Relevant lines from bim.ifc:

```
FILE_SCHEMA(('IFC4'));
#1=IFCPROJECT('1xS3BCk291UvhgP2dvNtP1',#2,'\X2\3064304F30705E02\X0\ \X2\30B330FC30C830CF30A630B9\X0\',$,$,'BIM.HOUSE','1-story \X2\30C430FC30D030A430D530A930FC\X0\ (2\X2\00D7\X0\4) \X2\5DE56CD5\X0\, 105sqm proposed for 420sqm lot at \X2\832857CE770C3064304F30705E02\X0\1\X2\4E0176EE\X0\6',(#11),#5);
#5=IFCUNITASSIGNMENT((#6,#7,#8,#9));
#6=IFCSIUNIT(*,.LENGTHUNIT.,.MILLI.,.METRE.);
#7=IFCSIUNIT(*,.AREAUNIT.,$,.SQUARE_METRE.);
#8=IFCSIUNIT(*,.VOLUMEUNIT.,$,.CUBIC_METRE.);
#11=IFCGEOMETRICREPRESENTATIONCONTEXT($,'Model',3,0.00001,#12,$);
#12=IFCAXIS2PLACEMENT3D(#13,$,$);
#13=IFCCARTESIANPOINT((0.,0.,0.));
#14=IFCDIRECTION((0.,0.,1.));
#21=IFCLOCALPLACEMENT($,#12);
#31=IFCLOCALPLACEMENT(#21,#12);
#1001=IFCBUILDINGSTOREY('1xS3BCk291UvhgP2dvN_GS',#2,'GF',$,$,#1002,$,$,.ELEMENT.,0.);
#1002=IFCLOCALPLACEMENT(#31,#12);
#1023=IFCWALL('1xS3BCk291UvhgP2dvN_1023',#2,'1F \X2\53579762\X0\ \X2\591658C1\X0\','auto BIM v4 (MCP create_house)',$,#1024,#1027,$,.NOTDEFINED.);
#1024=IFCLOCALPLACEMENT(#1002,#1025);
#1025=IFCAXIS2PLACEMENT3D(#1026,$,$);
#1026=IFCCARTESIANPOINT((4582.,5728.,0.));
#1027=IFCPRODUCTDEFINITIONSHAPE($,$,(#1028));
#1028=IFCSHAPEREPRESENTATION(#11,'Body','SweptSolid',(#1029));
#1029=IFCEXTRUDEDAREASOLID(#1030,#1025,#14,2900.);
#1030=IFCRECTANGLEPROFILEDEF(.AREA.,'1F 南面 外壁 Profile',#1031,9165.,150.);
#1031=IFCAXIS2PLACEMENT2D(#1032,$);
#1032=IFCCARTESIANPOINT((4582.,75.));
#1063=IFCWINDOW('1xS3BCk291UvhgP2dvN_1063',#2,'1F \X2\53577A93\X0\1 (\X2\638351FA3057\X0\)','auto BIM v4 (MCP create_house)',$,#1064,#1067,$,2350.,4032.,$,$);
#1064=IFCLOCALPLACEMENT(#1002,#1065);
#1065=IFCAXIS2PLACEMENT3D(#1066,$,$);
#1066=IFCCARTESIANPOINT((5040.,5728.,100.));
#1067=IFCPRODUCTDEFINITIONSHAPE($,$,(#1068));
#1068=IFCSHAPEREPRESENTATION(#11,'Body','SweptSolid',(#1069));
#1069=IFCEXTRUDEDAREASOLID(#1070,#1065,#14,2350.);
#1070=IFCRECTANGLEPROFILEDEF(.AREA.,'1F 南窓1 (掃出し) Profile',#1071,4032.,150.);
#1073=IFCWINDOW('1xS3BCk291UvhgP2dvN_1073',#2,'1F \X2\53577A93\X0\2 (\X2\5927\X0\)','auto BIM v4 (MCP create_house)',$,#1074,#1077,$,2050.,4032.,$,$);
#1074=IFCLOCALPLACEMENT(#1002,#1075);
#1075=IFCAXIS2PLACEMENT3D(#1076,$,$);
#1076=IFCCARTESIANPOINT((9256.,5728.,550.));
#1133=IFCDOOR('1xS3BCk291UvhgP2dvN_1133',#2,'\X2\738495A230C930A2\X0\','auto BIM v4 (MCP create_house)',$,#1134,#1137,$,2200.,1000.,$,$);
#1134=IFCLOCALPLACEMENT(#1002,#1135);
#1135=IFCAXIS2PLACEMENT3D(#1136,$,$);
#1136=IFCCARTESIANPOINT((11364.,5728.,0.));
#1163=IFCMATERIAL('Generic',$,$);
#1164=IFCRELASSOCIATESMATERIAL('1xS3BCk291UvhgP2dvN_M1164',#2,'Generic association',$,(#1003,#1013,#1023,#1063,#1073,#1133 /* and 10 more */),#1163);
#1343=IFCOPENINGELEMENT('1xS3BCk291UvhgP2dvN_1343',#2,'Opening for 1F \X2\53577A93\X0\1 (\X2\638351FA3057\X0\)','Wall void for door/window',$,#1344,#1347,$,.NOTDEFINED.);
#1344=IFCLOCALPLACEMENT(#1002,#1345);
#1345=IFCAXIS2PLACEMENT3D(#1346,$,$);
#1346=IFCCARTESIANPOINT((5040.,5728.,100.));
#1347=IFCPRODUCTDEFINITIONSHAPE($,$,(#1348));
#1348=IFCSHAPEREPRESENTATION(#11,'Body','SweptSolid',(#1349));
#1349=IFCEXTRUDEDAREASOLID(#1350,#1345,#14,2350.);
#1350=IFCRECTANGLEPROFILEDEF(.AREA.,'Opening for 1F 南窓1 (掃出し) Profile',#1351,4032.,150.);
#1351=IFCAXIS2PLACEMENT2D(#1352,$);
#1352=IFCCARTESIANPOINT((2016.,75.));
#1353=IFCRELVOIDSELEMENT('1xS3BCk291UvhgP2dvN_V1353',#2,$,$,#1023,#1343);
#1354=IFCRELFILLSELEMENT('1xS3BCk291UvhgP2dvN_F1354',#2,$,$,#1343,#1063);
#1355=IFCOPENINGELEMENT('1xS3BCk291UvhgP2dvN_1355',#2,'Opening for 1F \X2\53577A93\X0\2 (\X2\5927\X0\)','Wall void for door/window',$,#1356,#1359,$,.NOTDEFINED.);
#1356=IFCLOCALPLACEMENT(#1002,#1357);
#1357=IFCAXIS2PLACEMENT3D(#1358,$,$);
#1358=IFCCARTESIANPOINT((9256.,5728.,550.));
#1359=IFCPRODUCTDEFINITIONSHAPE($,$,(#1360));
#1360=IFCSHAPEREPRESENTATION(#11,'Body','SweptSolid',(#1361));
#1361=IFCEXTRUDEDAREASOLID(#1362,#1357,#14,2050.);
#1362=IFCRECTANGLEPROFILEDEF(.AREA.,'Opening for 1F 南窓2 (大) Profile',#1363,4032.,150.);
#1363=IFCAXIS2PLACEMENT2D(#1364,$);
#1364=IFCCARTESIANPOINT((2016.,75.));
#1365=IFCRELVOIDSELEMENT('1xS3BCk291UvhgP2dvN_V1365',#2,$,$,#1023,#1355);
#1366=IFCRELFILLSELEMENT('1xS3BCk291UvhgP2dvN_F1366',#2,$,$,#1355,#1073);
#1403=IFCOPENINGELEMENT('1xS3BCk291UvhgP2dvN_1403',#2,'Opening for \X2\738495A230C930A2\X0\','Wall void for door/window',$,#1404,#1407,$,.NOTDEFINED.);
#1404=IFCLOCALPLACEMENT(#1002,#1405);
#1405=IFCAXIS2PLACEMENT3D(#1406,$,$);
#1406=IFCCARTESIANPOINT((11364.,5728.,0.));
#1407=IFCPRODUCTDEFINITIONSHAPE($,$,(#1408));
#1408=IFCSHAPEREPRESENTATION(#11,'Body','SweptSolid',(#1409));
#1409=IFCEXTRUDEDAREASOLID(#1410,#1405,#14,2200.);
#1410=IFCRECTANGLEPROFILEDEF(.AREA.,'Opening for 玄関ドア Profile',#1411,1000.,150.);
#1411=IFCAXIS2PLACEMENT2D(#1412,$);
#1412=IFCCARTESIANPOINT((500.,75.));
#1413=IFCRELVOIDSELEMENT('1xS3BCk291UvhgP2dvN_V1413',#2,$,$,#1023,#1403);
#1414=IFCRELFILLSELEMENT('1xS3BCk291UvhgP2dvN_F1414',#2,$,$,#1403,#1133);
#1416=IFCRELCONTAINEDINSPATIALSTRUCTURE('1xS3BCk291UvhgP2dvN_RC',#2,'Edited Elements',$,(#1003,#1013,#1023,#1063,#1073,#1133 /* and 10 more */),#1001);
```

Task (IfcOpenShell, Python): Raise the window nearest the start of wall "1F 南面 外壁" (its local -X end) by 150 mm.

```python
import numpy as np
import ifcopenshell
import ifcopenshell.api.geometry
import ifcopenshell.util.placement
import ifcopenshell.util.unit

model = ifcopenshell.open("bim.ifc")
unit_scale = ifcopenshell.util.unit.calculate_unit_scale(model)

window = model.by_guid("1xS3BCk291UvhgP2dvN_1063")
opening = window.FillsVoids[0].RelatingOpeningElement
dz = 150.0

shift = np.array([0.0, 0.0, dz])
# The window is not placed relative to its opening, so move both.
for product in (opening, window):
    matrix = ifcopenshell.util.placement.get_local_placement(product.ObjectPlacement)
    matrix[:3, 3] += shift
    ifcopenshell.api.geometry.edit_object_placement(model, product=product, matrix=matrix, is_si=False)

print(f"moved by {dz * unit_scale:+.3f} m")

model.write("bim_v2.ifc")
```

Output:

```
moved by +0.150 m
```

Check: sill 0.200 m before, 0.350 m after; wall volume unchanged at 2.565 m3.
